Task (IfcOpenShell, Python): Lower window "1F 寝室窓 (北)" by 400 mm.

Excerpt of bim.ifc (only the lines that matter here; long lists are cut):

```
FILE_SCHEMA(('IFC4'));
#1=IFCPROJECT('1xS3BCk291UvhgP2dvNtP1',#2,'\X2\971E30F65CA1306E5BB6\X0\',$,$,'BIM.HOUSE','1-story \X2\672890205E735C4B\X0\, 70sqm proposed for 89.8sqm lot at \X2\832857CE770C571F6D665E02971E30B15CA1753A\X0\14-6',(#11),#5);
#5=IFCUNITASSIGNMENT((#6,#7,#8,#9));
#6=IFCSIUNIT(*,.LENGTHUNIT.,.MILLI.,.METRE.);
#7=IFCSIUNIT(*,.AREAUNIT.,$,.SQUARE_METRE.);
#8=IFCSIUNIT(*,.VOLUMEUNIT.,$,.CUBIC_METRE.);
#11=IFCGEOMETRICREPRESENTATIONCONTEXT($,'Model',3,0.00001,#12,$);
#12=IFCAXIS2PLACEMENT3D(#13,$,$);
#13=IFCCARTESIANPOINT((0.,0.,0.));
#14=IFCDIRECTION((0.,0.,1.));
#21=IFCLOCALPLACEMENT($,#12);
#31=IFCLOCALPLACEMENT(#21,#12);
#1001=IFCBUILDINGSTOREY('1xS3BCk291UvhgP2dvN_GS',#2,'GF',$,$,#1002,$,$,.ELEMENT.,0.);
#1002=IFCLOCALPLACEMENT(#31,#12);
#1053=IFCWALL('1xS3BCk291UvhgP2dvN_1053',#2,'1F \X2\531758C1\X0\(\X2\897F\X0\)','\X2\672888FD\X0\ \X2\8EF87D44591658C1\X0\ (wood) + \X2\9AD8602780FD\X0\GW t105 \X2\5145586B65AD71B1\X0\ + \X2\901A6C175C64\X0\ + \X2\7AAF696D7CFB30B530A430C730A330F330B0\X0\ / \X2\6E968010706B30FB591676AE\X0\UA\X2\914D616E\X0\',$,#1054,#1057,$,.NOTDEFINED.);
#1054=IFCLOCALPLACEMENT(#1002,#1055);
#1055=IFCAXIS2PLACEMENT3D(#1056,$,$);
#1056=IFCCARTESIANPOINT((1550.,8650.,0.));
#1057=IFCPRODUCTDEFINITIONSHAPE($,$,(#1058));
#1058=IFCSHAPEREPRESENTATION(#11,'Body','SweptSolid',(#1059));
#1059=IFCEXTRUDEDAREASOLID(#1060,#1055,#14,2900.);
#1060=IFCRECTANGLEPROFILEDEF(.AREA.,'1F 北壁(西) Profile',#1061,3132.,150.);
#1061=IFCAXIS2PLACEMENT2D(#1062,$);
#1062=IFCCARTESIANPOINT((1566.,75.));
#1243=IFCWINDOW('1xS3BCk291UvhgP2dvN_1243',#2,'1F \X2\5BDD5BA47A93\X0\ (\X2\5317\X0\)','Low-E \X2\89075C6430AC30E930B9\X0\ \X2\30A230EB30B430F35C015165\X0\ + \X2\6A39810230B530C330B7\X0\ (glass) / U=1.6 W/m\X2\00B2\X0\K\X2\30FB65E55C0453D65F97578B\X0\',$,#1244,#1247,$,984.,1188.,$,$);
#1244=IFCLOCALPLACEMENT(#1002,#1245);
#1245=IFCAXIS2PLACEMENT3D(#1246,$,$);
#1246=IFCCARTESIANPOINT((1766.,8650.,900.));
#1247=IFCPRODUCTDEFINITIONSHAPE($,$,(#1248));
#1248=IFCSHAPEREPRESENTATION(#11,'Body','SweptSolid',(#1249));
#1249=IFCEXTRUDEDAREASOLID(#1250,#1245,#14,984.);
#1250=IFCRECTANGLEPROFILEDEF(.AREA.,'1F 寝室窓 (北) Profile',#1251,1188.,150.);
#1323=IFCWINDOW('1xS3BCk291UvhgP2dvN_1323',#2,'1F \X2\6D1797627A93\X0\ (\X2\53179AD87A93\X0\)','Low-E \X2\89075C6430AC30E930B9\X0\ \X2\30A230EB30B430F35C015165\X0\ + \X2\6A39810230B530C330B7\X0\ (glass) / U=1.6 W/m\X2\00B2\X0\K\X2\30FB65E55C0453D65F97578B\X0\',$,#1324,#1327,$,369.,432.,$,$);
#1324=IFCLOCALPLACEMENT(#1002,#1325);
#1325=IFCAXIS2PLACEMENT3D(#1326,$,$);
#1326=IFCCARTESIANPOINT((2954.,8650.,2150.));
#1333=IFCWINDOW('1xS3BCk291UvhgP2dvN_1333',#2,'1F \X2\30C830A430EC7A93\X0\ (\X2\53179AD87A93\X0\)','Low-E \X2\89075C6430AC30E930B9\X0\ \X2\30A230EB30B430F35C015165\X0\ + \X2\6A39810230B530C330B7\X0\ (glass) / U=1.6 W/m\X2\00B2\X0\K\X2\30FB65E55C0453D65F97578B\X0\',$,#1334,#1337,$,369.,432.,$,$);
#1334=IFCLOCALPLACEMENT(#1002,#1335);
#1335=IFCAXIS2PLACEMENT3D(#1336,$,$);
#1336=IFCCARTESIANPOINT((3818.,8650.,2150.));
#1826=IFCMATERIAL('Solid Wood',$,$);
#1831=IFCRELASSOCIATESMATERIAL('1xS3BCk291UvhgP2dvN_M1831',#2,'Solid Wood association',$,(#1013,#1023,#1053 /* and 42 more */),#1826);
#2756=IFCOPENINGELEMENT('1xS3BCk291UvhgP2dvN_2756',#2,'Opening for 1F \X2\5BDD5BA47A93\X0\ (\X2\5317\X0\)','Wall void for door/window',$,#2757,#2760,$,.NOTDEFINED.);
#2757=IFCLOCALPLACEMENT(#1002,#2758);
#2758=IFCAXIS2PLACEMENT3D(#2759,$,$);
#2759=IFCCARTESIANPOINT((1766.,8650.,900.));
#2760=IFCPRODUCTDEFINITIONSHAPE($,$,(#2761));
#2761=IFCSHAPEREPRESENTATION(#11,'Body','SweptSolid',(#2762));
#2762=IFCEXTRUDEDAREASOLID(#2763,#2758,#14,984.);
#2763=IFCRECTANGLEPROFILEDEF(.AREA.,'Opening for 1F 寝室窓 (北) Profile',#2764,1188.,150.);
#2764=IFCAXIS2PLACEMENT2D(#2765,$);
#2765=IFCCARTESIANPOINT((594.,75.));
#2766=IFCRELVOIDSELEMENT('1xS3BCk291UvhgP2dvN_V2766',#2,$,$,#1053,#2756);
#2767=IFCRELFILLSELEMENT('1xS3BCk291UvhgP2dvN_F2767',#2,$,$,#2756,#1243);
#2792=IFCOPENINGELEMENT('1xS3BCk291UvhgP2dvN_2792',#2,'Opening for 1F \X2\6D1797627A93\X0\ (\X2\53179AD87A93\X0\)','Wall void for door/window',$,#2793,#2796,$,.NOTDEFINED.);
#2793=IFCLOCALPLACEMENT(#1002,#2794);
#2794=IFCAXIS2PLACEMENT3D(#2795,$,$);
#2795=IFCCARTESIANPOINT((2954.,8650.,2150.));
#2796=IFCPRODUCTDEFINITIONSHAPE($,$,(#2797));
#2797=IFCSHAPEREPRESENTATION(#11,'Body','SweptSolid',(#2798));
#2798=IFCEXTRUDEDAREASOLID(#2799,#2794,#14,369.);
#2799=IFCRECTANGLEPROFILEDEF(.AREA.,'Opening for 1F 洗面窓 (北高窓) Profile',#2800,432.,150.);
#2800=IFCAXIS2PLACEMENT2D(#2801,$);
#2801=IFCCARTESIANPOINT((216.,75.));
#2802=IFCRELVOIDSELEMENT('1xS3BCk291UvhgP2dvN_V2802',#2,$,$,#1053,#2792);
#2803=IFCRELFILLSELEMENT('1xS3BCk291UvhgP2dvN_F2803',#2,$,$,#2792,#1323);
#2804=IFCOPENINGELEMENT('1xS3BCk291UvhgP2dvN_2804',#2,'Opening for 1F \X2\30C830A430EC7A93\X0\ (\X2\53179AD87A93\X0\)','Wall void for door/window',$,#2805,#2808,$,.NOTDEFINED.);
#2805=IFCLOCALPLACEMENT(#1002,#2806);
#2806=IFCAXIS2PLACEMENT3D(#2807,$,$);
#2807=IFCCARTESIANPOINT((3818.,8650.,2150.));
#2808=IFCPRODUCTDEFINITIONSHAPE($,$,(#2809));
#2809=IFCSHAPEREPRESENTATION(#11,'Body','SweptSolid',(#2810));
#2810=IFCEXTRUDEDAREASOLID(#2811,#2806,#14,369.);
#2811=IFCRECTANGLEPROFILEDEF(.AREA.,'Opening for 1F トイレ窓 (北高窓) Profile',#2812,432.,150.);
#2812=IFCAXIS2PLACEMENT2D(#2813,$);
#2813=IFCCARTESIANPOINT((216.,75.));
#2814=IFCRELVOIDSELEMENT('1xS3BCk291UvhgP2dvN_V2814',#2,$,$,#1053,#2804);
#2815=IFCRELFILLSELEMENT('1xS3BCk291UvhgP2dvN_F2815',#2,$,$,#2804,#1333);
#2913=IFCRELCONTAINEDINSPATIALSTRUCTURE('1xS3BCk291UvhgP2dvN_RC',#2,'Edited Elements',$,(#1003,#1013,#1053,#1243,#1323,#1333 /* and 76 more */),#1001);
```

```python
import numpy as np
import ifcopenshell
import ifcopenshell.api.geometry
import ifcopenshell.util.placement
import ifcopenshell.util.unit

model = ifcopenshell.open("bim.ifc")
unit_scale = ifcopenshell.util.unit.calculate_unit_scale(model)

window = model.by_guid("1xS3BCk291UvhgP2dvN_1243")
opening = window.FillsVoids[0].RelatingOpeningElement
dz = -400.0

shift = np.array([0.0, 0.0, dz])
# The window is not placed relative to its opening, so move both.
for product in (opening, window):
    matrix = ifcopenshell.util.placement.get_local_placement(product.ObjectPlacement)
    matrix[:3, 3] += shift
    ifcopenshell.api.geometry.edit_object_placement(model, product=product, matrix=matrix, is_si=False)

print(f"moved by {dz * unit_scale:+.3f} m")

model.write("bim_v2.ifc")
```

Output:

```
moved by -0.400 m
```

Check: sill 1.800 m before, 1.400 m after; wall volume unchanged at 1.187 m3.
